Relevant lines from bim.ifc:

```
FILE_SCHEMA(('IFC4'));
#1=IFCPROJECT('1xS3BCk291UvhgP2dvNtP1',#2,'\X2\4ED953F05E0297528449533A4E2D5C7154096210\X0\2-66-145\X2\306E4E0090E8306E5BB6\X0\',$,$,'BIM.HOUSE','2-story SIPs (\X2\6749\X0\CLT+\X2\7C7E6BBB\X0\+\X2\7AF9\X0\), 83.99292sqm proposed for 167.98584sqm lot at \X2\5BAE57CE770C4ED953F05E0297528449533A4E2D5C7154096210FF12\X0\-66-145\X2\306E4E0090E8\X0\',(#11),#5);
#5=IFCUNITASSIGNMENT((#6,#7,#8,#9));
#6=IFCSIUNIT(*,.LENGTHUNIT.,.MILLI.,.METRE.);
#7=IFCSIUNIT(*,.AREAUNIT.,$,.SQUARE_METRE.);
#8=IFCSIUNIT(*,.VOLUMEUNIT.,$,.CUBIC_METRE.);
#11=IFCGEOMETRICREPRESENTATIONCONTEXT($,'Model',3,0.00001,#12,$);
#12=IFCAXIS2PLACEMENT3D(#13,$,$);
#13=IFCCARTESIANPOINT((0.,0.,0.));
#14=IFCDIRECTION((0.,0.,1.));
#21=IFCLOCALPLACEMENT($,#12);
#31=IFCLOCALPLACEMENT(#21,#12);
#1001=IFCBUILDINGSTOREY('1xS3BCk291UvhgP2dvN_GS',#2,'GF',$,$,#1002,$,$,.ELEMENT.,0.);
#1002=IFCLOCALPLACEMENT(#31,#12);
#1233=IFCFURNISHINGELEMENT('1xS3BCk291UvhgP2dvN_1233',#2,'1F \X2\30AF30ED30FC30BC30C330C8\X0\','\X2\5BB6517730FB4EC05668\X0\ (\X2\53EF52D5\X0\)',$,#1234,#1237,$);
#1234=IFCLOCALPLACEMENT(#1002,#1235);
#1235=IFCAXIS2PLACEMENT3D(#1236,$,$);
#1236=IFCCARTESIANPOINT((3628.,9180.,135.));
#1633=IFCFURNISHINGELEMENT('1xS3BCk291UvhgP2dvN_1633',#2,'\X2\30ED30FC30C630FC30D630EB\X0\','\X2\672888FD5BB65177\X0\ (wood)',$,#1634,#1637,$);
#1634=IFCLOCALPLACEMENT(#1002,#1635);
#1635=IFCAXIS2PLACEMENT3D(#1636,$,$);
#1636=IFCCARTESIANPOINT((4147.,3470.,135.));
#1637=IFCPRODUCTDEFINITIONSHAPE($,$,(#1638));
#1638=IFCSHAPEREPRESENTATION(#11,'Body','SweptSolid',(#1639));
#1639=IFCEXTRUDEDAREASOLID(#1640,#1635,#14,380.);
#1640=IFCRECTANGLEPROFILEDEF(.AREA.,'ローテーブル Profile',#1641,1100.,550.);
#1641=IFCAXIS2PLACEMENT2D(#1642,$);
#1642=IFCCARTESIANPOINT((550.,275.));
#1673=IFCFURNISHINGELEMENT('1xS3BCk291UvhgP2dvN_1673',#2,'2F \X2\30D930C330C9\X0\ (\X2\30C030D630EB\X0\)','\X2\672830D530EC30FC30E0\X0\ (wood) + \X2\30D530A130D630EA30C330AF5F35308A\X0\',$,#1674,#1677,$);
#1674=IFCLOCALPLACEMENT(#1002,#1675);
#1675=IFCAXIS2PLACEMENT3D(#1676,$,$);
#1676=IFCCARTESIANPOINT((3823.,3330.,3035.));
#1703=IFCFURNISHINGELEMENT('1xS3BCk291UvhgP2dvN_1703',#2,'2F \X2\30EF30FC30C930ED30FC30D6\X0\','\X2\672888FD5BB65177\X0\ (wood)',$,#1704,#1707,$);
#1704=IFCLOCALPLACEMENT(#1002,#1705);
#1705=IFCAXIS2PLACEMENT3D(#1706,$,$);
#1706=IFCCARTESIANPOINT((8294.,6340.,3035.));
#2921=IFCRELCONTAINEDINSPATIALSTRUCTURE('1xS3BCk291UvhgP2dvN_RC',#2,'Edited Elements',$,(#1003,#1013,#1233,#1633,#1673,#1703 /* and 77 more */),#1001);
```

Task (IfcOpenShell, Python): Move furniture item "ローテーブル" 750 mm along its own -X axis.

```python
import ifcopenshell
import ifcopenshell.api.geometry
import ifcopenshell.util.placement
import ifcopenshell.util.unit

model = ifcopenshell.open("bim.ifc")
unit_scale = ifcopenshell.util.unit.calculate_unit_scale(model)

item = model.by_id(1633)
matrix = ifcopenshell.util.placement.get_local_placement(item.ObjectPlacement)
matrix[:3, 3] -= matrix[:3, 0] * 0.75 / unit_scale
ifcopenshell.api.geometry.edit_object_placement(model, product=item, matrix=matrix, is_si=False)

print(ifcopenshell.util.placement.get_local_placement(item.ObjectPlacement).round(3) + 0.0)

model.write("bim_rev.ifc")
```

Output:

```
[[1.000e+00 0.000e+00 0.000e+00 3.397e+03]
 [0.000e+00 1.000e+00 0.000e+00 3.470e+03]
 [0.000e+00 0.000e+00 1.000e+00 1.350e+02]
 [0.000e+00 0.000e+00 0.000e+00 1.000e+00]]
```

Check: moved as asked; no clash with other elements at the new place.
